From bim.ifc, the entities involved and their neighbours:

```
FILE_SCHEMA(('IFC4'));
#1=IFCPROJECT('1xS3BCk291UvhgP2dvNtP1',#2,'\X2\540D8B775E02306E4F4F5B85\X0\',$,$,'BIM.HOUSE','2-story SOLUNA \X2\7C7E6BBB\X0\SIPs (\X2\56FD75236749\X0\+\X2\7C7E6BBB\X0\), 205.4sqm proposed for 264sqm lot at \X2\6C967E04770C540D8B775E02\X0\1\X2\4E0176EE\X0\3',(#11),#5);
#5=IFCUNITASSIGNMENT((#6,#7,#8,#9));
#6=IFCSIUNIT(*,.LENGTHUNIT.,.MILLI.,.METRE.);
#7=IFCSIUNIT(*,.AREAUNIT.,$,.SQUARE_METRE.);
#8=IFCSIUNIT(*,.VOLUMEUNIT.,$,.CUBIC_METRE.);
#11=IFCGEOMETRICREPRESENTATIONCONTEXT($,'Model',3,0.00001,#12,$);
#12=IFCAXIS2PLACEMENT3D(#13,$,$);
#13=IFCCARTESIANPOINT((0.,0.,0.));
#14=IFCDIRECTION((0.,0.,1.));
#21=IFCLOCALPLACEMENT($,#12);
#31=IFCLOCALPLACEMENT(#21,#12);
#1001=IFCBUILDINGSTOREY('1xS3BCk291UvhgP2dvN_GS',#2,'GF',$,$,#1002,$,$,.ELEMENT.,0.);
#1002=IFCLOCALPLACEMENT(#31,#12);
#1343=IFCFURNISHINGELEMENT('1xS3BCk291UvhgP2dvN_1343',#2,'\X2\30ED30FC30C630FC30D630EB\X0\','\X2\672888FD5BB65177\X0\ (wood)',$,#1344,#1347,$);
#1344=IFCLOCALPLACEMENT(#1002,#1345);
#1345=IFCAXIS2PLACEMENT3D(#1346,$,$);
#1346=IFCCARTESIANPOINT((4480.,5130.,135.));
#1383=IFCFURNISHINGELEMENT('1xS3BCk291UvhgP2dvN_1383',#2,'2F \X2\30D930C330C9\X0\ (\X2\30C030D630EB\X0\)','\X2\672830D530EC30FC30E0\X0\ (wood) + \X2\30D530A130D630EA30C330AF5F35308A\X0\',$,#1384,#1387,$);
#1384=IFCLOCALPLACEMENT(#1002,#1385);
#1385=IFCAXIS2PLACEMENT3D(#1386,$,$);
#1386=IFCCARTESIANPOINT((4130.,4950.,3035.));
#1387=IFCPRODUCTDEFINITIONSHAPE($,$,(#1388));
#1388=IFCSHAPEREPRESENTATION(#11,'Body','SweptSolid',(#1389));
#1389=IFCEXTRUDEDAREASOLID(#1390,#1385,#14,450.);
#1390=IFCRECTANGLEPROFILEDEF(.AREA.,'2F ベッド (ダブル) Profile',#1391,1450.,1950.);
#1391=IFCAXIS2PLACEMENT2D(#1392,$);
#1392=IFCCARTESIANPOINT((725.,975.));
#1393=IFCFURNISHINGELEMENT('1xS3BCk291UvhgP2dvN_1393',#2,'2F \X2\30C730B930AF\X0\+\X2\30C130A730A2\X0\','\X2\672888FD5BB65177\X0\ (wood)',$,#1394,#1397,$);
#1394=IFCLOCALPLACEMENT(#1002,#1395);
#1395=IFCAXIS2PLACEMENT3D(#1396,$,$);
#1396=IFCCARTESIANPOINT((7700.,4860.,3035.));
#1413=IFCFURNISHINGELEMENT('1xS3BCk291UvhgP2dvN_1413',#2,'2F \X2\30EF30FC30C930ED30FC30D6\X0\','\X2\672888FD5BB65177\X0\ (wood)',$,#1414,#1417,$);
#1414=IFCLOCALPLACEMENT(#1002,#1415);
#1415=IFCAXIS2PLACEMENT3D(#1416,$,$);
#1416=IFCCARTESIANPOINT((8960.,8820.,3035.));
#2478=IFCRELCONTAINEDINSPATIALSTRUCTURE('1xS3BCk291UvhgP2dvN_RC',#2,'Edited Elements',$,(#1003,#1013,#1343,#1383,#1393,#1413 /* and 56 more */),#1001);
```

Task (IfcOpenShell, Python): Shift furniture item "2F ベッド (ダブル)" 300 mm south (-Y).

```python
import ifcopenshell
import ifcopenshell.api.geometry
import ifcopenshell.util.placement
import ifcopenshell.util.unit

model = ifcopenshell.open("bim.ifc")
unit_scale = ifcopenshell.util.unit.calculate_unit_scale(model)

item = model.by_guid("1xS3BCk291UvhgP2dvN_1383")
matrix = ifcopenshell.util.placement.get_local_placement(item.ObjectPlacement)
matrix[1, 3] -= 0.3 / unit_scale
ifcopenshell.api.geometry.edit_object_placement(model, product=item, matrix=matrix, is_si=False)

print(ifcopenshell.util.placement.get_local_placement(item.ObjectPlacement).round(3) + 0.0)

model.write("bim_updated.ifc")
```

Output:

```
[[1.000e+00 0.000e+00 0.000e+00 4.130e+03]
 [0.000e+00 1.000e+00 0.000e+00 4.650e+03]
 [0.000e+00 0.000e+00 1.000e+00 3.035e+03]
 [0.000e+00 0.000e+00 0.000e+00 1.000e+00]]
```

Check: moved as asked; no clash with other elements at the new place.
